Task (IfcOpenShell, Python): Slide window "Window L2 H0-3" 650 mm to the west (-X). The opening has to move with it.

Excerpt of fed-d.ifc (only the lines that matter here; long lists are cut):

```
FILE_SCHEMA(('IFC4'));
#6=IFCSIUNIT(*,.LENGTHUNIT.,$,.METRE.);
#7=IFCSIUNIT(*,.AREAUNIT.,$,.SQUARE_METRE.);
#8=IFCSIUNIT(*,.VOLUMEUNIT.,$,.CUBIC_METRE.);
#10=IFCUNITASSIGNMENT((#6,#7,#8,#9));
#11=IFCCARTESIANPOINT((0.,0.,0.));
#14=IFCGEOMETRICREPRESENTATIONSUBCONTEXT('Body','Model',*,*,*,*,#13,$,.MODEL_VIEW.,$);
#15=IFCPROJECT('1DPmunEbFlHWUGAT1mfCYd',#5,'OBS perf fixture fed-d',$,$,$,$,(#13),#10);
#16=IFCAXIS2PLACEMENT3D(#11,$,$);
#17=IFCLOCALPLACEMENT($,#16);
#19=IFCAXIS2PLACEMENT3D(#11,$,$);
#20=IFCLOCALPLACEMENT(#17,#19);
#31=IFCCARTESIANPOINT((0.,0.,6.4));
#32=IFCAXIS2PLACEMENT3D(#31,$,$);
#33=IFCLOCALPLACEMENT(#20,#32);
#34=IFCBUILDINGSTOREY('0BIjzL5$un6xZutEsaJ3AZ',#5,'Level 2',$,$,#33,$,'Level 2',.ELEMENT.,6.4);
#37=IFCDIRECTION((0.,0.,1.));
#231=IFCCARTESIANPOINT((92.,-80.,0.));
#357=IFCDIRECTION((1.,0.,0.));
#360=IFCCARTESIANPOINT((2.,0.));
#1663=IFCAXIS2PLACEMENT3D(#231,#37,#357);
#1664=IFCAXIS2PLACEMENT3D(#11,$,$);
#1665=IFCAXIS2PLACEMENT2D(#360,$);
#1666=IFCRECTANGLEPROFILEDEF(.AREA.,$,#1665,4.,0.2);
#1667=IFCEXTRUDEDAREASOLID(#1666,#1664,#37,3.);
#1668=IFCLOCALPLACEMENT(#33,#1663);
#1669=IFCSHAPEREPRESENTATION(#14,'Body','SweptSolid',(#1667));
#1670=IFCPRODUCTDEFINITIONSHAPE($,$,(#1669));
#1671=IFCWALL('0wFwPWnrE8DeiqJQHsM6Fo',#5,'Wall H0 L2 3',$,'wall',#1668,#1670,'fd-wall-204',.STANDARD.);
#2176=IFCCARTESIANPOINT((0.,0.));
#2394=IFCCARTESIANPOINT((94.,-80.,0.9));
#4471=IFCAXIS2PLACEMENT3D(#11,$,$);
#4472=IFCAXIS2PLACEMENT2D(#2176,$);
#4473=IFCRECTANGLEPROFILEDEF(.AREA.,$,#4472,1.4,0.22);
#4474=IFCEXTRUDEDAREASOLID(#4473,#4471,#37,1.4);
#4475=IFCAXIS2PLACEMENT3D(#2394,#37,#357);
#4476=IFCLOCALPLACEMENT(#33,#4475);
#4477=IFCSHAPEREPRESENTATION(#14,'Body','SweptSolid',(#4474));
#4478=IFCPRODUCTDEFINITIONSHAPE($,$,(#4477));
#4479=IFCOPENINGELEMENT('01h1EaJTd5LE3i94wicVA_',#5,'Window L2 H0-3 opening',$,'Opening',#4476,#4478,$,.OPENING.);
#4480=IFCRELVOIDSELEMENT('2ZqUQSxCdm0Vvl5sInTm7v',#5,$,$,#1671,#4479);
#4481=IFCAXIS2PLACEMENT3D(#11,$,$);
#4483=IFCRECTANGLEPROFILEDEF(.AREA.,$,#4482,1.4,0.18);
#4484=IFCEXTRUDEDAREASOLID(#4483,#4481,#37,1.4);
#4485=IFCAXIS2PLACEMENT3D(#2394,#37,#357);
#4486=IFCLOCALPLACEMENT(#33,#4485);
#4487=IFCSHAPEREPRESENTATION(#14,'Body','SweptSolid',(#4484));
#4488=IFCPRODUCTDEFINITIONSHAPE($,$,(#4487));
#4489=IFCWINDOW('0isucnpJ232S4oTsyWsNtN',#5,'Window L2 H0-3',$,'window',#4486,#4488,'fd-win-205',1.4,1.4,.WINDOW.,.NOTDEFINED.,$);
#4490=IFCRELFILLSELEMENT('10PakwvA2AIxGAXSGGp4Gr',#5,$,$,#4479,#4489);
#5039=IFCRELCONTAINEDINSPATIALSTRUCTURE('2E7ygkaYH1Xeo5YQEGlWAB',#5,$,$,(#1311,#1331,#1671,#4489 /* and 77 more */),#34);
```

```python
import ifcopenshell
import ifcopenshell.api.geometry
import ifcopenshell.util.placement

model = ifcopenshell.open("fed-d.ifc")

window = model.by_guid("0isucnpJ232S4oTsyWsNtN")
opening = window.FillsVoids[0].RelatingOpeningElement
wall = opening.VoidsElements[0].RelatingBuildingElement

wall_matrix = ifcopenshell.util.placement.get_local_placement(wall.ObjectPlacement)
shift = wall_matrix[:3, 0] * -0.65
before = ifcopenshell.util.placement.get_local_placement(window.ObjectPlacement)[:3, 3].copy()

# The window is not placed relative to its opening, so move both.
for product in (opening, window):
    matrix = ifcopenshell.util.placement.get_local_placement(product.ObjectPlacement)
    matrix[:3, 3] += shift
    ifcopenshell.api.geometry.edit_object_placement(model, product=product, matrix=matrix, is_si=False)

after = ifcopenshell.util.placement.get_local_placement(window.ObjectPlacement)[:3, 3]
print("window moved by", (after - before).round(3) + 0.0)

model.write("fed-d_v2.ifc")
```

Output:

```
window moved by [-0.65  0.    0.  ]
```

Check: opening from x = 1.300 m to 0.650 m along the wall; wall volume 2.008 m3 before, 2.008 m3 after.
